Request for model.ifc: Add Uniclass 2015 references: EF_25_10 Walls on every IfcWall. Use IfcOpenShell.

First a look at what the model holds.

```python
import ifcopenshell

model = ifcopenshell.open("model.ifc")
print(model.schema)
print("classifications:", [c.Name for c in model.by_type("IfcClassification")])
for ifc_class in ("IfcDoor", "IfcRoof", "IfcStair", "IfcWall", "IfcWindow"):
    print(ifc_class, len(model.by_type(ifc_class)))
```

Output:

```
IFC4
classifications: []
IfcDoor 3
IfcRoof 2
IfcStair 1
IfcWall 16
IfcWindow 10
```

```python
import ifcopenshell
import ifcopenshell.api.classification

model = ifcopenshell.open("model.ifc")

system = ifcopenshell.api.classification.add_classification(model, classification="Uniclass 2015")

codes = {
    "IfcWall": ("EF_25_10", "Walls"),
}
for ifc_class, (code, name) in codes.items():
    products = model.by_type(ifc_class)
    ifcopenshell.api.classification.add_reference(
        model, products=products, classification=system, identification=code, name=name
    )
    print(code, len(products))

model.write("model_v2.ifc")
```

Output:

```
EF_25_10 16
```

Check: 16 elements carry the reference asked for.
